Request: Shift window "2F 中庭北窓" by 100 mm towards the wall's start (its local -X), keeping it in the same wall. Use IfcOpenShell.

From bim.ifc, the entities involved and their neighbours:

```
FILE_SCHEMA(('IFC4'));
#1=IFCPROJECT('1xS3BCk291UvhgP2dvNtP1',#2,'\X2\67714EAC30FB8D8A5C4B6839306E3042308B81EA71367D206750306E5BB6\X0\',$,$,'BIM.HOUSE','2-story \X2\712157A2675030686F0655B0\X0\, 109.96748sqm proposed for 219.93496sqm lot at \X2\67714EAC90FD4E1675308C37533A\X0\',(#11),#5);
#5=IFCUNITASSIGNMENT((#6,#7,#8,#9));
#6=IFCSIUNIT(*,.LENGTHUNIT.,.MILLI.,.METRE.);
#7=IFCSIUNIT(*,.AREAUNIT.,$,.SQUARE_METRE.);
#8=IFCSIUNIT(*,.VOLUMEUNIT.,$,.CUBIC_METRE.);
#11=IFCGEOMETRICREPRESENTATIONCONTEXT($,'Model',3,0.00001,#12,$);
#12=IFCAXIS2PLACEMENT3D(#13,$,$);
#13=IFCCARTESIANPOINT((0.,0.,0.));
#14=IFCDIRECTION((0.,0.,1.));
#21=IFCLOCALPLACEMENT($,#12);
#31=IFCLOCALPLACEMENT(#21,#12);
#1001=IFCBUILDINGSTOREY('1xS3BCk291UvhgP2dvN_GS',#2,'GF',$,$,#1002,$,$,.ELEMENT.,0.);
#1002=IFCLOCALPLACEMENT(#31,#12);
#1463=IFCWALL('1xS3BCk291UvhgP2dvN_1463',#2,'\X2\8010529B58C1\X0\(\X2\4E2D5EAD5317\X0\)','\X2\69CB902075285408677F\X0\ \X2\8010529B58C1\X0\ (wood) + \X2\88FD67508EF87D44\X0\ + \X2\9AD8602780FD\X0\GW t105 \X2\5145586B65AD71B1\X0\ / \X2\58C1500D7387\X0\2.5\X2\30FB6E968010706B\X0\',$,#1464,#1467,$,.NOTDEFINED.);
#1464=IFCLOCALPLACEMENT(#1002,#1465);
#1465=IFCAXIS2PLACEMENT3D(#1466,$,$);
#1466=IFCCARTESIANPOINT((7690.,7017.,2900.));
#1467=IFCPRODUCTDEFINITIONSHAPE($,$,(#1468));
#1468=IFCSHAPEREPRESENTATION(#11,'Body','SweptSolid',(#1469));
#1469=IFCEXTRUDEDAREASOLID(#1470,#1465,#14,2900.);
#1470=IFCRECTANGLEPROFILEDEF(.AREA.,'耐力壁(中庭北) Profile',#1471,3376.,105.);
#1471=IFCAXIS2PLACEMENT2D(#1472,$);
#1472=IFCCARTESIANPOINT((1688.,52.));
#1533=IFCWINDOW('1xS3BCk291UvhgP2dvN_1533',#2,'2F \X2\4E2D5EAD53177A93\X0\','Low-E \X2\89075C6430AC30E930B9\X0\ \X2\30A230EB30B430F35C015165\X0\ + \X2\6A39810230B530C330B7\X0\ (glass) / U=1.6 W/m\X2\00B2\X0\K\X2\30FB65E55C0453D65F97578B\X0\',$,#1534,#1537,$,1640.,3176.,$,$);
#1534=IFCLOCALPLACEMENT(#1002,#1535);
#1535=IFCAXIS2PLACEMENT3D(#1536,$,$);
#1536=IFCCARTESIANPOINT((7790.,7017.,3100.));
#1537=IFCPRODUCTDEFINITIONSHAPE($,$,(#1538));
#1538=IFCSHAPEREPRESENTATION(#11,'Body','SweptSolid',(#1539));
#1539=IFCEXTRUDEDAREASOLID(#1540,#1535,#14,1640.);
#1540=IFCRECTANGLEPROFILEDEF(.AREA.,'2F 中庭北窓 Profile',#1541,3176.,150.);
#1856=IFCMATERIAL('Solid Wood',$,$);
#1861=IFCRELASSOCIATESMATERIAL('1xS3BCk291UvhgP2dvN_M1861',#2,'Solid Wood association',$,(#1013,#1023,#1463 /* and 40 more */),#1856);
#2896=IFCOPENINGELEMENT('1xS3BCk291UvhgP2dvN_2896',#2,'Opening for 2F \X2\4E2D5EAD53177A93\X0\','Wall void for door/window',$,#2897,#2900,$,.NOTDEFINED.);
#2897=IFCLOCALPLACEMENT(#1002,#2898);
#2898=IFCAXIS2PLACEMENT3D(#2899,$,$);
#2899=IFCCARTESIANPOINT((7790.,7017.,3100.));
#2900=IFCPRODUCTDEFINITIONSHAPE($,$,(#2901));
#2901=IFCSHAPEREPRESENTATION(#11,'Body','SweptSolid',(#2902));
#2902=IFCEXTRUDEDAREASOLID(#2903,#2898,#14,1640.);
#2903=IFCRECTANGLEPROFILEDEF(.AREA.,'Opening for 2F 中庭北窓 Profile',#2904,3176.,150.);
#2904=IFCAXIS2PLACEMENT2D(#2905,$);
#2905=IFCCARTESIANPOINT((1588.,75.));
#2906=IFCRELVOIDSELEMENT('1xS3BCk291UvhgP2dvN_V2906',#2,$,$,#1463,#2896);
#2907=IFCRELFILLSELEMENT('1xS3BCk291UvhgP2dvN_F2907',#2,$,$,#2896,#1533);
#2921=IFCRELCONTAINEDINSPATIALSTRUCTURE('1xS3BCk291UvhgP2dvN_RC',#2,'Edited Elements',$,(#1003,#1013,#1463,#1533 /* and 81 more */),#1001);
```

```python
import ifcopenshell
import ifcopenshell.api.geometry
import ifcopenshell.util.placement
import ifcopenshell.util.unit

model = ifcopenshell.open("bim.ifc")
unit_scale = ifcopenshell.util.unit.calculate_unit_scale(model)

window = model.by_guid("1xS3BCk291UvhgP2dvN_1533")
opening = window.FillsVoids[0].RelatingOpeningElement
wall = opening.VoidsElements[0].RelatingBuildingElement

wall_matrix = ifcopenshell.util.placement.get_local_placement(wall.ObjectPlacement)
shift = wall_matrix[:3, 0] * -0.1 / unit_scale
before = ifcopenshell.util.placement.get_local_placement(window.ObjectPlacement)[:3, 3].copy()

# The window is not placed relative to its opening, so move both.
for product in (opening, window):
    matrix = ifcopenshell.util.placement.get_local_placement(product.ObjectPlacement)
    matrix[:3, 3] += shift
    ifcopenshell.api.geometry.edit_object_placement(model, product=product, matrix=matrix, is_si=False)

after = ifcopenshell.util.placement.get_local_placement(window.ObjectPlacement)[:3, 3]
print("window moved by", (after - before).round(3) + 0.0)

model.write("bim_rev.ifc")
```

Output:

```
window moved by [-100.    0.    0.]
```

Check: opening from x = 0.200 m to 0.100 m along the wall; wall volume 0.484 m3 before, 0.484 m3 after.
